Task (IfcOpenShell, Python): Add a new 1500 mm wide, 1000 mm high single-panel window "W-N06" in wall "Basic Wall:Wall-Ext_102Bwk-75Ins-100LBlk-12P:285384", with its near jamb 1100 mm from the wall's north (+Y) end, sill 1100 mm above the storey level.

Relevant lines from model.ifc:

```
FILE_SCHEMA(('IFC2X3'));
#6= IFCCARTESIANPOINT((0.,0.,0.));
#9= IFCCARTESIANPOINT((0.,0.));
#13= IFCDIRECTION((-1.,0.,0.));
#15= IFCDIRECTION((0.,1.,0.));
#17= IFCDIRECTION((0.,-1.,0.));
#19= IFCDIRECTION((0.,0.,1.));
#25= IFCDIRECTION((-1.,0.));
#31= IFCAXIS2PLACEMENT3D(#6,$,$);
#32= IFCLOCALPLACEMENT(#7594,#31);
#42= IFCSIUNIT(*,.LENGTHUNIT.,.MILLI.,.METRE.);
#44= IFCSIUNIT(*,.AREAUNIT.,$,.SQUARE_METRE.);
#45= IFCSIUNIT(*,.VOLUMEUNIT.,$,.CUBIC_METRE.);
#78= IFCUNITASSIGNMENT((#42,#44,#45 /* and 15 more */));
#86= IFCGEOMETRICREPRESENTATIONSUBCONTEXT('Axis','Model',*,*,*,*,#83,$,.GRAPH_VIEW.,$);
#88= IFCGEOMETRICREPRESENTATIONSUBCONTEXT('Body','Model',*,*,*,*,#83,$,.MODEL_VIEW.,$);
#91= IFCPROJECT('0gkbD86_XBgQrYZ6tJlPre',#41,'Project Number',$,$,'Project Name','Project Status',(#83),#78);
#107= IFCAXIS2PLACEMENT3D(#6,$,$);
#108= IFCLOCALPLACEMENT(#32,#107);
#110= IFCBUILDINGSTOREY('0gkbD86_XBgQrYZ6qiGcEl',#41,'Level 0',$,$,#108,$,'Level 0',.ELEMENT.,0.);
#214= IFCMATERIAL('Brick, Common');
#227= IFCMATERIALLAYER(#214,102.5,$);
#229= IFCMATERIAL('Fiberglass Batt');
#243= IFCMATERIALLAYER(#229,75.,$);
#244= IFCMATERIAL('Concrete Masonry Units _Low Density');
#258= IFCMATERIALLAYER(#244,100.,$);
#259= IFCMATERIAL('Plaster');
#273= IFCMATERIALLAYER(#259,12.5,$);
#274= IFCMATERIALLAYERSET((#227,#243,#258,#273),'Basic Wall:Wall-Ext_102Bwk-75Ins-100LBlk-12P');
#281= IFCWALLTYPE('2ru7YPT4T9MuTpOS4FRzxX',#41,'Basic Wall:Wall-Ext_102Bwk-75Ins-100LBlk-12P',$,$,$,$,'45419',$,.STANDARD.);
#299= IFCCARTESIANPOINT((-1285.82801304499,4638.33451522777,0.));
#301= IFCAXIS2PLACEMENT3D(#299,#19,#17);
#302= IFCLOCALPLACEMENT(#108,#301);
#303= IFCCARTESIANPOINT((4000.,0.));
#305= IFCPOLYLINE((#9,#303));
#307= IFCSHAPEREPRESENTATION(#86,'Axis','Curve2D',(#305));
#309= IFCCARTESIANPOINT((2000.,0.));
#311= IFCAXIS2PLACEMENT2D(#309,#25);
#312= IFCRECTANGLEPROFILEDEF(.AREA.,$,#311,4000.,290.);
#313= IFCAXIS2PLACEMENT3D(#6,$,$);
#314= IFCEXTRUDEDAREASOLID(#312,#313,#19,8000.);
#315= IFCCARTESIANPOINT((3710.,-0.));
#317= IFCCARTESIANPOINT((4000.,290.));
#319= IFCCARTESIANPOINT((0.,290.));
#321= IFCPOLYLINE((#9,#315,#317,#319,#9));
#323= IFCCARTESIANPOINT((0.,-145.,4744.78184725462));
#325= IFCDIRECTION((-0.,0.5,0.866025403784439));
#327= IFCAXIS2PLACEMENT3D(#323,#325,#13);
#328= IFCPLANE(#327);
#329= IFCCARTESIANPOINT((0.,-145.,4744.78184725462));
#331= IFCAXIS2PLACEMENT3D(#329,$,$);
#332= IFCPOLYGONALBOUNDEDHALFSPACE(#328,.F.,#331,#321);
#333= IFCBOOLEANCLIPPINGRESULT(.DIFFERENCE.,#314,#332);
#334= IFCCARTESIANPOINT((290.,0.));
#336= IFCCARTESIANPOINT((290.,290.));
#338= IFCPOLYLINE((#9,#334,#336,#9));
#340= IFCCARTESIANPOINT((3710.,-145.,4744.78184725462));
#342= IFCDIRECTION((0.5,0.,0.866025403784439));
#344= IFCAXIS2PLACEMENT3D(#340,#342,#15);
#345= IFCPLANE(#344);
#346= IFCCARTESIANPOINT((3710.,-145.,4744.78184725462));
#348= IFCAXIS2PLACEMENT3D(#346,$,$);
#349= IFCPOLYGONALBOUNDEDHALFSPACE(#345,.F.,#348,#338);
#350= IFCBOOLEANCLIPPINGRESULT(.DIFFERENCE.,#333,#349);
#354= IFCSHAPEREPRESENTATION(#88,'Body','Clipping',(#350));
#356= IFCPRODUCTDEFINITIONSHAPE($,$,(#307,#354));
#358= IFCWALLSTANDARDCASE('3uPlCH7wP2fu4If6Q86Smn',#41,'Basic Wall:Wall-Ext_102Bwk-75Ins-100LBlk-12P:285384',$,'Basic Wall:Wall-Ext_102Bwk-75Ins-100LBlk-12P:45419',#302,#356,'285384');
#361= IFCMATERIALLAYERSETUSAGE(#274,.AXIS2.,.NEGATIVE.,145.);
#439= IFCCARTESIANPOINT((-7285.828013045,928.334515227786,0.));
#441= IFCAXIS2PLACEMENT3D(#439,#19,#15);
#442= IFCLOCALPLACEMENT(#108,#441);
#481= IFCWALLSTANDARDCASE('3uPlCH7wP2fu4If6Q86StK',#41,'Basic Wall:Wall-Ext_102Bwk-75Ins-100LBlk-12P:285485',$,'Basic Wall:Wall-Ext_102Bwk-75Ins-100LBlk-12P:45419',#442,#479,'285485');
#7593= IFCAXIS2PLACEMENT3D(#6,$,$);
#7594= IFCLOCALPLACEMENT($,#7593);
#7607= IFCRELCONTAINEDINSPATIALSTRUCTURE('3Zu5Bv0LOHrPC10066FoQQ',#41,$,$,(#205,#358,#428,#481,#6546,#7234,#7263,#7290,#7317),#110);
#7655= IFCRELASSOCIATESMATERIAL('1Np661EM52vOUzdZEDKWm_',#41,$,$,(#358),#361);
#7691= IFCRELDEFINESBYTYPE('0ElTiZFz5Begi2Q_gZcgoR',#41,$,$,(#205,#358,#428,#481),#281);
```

```python
import numpy as np
import ifcopenshell
import ifcopenshell.api.feature
import ifcopenshell.api.geometry
import ifcopenshell.api.root
import ifcopenshell.api.spatial
import ifcopenshell.api.type
import ifcopenshell.geom
import ifcopenshell.util.element
import ifcopenshell.util.placement
import ifcopenshell.util.representation
import ifcopenshell.util.shape
import ifcopenshell.util.unit

model = ifcopenshell.open("model.ifc")
unit_scale = ifcopenshell.util.unit.calculate_unit_scale(model)
settings = ifcopenshell.geom.settings()


def volume(element):
    """Net volume in cubic metres, openings subtracted."""
    shape = ifcopenshell.geom.create_shape(settings, element)
    return ifcopenshell.util.shape.get_volume(shape.geometry)


wall = model.by_guid("3uPlCH7wP2fu4If6Q86Smn")
storey = ifcopenshell.util.element.get_container(wall, ifc_class="IfcBuildingStorey")
context = ifcopenshell.util.representation.get_context(model, "Model", "Body", "MODEL_VIEW")
before = volume(wall)

width, height, from_end, sill = 1.5, 1, 1.1, 1.1  # metres

# The wall runs along its own X axis, and the end named is its -X end.
wall_shape = ifcopenshell.geom.create_shape(settings, wall)
x, y, z = ifcopenshell.util.shape.get_vertices(wall_shape.geometry).T
start = x.min() + from_end
face, thickness = float(y.min()), float(y.max() - y.min())
wall_matrix = ifcopenshell.util.placement.get_local_placement(wall.ObjectPlacement)
level = ifcopenshell.util.placement.get_local_placement(storey.ObjectPlacement)[2, 3]


def in_wall(x, y):
    """Placement at x, y metres in the wall's axes, at sill height."""
    matrix = wall_matrix.copy()
    matrix[:, 3] = wall_matrix @ np.array([x / unit_scale, y / unit_scale, 0.0, 1.0])
    matrix[2, 3] = level + sill / unit_scale
    return matrix


# Opening: a box that overshoots both wall faces by 50 mm.
opening = ifcopenshell.api.root.create_entity(model, ifc_class="IfcOpeningElement")
box = ifcopenshell.api.geometry.add_wall_representation(
    model, context=context, length=width, height=height, thickness=thickness + 0.1
)
ifcopenshell.api.geometry.assign_representation(model, product=opening, representation=box)
ifcopenshell.api.geometry.edit_object_placement(model, product=opening, matrix=in_wall(start, face - 0.05), is_si=False)
ifcopenshell.api.feature.add_feature(model, feature=opening, element=wall)

window = ifcopenshell.api.root.create_entity(model, ifc_class="IfcWindow", name="W-N06")
window.OverallWidth, window.OverallHeight = width / unit_scale, height / unit_scale
body = ifcopenshell.api.geometry.add_window_representation(
    model,
    context=context,
    overall_width=window.OverallWidth,
    overall_height=window.OverallHeight,
    partition_type="SINGLE_PANEL",
)
ifcopenshell.api.geometry.assign_representation(model, product=window, representation=body)
ifcopenshell.api.spatial.assign_container(model, products=[window], relating_structure=storey)
fills = ifcopenshell.api.feature.add_filling(model, opening=opening, element=window)
fills.OwnerHistory = window.OwnerHistory  # required in IFC2X3

# IFC2X3 keeps the operation on the window style.
style = ifcopenshell.api.root.create_entity(model, ifc_class="IfcWindowStyle", name="W-N06")
style.OperationType, style.ConstructionType = "SINGLE_PANEL", "NOTDEFINED"
style.ParameterTakesPrecedence = style.Sizeable = False
ifcopenshell.api.type.assign_type(model, related_objects=[window], relating_type=style)

# Centre the window in the wall's thickness.
ifcopenshell.api.geometry.edit_object_placement(model, product=window, matrix=in_wall(start, face), is_si=False)
window_shape = ifcopenshell.geom.create_shape(settings, window)
depth = ifcopenshell.util.shape.get_vertices(window_shape.geometry)[:, 1]
offset = face + thickness / 2 - (depth.min() + depth.max()) / 2
ifcopenshell.api.geometry.edit_object_placement(model, product=window, matrix=in_wall(start, offset), is_si=False)

after = volume(wall)

print(f"wall volume {before:.3f} -> {after:.3f} m3")

model.write("model_updated.ifc")
```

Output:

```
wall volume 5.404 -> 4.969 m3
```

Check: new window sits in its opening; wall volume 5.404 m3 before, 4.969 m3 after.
